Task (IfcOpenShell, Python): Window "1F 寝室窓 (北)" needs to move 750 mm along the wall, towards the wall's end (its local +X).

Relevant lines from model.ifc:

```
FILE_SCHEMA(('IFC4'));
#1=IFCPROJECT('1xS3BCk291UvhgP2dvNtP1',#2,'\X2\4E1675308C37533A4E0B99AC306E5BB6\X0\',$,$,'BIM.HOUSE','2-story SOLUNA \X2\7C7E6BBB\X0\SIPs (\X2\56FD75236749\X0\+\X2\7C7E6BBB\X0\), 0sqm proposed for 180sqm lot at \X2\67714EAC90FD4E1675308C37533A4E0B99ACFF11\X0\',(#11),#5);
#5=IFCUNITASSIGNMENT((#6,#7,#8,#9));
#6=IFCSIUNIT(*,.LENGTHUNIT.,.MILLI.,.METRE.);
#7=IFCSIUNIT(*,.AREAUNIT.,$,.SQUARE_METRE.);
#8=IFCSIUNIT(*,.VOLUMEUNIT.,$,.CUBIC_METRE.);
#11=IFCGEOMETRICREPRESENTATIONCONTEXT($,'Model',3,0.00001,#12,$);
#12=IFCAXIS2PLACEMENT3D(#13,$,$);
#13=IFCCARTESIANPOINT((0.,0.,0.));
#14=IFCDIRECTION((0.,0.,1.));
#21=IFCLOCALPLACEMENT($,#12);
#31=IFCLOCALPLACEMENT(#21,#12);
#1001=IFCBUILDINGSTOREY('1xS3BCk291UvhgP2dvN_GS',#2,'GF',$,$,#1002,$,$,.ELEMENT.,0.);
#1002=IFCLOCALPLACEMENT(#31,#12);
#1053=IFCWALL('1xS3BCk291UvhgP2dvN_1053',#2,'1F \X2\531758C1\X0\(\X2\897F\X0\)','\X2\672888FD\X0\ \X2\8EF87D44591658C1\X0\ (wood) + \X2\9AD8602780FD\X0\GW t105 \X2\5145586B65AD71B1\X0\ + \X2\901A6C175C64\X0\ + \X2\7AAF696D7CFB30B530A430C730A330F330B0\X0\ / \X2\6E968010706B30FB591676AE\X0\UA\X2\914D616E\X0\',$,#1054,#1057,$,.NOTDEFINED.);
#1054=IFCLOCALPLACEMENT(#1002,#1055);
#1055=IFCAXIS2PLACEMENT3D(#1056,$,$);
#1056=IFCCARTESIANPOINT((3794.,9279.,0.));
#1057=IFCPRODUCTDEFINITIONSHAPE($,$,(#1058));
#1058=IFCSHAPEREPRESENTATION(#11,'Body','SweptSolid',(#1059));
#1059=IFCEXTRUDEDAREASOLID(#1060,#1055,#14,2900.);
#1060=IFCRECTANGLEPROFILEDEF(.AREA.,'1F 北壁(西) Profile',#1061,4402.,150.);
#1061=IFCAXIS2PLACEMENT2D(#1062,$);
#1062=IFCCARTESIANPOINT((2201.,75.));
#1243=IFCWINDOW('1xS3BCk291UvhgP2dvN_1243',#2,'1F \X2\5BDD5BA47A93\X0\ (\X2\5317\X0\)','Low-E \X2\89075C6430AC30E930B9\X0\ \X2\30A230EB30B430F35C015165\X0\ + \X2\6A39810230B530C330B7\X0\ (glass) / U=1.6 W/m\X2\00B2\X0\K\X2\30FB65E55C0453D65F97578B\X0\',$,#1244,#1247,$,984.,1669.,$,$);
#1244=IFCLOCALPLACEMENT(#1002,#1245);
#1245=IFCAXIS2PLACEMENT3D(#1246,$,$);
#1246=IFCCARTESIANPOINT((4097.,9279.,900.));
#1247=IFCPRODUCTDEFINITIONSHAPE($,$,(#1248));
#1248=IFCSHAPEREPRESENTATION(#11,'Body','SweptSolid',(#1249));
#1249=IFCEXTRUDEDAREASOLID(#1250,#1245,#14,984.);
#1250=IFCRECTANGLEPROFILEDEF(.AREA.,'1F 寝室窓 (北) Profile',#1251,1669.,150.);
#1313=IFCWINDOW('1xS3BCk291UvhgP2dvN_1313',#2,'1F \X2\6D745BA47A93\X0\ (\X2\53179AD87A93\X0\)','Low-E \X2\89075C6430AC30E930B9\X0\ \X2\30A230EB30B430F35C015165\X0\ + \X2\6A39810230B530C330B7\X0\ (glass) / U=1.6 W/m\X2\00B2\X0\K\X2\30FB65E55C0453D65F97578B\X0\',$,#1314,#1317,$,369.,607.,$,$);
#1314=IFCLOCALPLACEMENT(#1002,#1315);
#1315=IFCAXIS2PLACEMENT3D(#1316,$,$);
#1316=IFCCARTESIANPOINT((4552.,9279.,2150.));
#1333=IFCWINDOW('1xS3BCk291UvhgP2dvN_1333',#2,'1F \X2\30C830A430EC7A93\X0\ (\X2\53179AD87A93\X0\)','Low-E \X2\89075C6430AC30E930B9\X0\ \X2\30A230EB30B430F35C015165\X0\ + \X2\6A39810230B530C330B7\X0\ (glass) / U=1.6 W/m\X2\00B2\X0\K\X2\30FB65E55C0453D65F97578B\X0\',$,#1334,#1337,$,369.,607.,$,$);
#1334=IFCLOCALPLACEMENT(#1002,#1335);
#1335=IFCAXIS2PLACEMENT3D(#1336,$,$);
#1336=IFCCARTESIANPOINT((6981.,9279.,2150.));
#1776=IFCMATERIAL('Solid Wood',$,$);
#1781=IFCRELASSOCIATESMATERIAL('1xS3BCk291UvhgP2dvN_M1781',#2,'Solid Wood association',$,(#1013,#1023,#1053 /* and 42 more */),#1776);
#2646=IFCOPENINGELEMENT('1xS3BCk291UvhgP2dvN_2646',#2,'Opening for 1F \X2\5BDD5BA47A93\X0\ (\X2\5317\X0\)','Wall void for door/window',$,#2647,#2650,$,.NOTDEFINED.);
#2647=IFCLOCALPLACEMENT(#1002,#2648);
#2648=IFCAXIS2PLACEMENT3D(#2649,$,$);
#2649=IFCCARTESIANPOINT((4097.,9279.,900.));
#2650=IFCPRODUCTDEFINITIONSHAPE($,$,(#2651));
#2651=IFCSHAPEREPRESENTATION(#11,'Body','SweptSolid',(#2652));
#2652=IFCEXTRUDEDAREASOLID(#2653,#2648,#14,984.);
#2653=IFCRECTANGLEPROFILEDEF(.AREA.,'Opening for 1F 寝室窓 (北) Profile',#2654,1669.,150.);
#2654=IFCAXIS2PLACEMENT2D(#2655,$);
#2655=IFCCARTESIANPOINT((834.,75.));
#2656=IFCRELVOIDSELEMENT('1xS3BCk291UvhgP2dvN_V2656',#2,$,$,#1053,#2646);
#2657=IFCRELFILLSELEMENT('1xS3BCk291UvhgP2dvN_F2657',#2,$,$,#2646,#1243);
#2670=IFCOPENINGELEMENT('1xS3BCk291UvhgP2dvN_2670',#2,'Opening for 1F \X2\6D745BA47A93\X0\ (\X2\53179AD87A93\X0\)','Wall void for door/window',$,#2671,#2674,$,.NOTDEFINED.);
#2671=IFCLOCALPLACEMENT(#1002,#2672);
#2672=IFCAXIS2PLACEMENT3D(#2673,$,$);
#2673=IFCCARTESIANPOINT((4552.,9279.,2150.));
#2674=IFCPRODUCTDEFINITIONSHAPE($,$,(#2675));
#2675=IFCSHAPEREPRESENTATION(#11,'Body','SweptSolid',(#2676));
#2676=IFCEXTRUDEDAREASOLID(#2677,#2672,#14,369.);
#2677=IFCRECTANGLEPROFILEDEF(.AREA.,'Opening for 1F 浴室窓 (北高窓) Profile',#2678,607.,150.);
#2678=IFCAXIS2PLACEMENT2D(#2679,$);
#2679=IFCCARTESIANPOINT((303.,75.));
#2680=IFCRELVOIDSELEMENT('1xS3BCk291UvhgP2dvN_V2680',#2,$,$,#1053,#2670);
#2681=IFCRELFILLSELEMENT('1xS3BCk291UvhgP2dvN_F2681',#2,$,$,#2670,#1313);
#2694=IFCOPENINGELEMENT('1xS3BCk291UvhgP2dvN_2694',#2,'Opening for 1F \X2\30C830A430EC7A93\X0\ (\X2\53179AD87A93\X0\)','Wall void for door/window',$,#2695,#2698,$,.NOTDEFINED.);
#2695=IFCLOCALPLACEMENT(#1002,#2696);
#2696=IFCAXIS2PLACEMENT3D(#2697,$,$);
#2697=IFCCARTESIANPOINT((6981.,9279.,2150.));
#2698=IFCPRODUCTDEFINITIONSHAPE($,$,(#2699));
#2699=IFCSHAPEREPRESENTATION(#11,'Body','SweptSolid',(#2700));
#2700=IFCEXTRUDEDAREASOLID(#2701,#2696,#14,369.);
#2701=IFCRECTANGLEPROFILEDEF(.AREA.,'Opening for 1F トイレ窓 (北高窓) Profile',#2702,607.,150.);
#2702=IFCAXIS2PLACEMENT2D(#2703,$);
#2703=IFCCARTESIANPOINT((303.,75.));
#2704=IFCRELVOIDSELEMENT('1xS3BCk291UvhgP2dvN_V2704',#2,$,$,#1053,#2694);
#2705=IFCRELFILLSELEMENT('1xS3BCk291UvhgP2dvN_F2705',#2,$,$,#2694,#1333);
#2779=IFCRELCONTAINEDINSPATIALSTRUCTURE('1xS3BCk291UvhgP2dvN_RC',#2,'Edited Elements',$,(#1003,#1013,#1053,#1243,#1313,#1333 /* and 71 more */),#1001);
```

```python
import ifcopenshell
import ifcopenshell.api.geometry
import ifcopenshell.util.placement
import ifcopenshell.util.unit

model = ifcopenshell.open("model.ifc")
unit_scale = ifcopenshell.util.unit.calculate_unit_scale(model)

window = model.by_guid("1xS3BCk291UvhgP2dvN_1243")
opening = window.FillsVoids[0].RelatingOpeningElement
wall = opening.VoidsElements[0].RelatingBuildingElement

wall_matrix = ifcopenshell.util.placement.get_local_placement(wall.ObjectPlacement)
shift = wall_matrix[:3, 0] * 0.75 / unit_scale
before = ifcopenshell.util.placement.get_local_placement(window.ObjectPlacement)[:3, 3].copy()

# The window is not placed relative to its opening, so move both.
for product in (opening, window):
    matrix = ifcopenshell.util.placement.get_local_placement(product.ObjectPlacement)
    matrix[:3, 3] += shift
    ifcopenshell.api.geometry.edit_object_placement(model, product=product, matrix=matrix, is_si=False)

after = ifcopenshell.util.placement.get_local_placement(window.ObjectPlacement)[:3, 3]
print("window moved by", (after - before).round(3) + 0.0)

model.write("model_updated.ifc")
```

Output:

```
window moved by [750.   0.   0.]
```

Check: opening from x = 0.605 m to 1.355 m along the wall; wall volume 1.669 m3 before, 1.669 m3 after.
